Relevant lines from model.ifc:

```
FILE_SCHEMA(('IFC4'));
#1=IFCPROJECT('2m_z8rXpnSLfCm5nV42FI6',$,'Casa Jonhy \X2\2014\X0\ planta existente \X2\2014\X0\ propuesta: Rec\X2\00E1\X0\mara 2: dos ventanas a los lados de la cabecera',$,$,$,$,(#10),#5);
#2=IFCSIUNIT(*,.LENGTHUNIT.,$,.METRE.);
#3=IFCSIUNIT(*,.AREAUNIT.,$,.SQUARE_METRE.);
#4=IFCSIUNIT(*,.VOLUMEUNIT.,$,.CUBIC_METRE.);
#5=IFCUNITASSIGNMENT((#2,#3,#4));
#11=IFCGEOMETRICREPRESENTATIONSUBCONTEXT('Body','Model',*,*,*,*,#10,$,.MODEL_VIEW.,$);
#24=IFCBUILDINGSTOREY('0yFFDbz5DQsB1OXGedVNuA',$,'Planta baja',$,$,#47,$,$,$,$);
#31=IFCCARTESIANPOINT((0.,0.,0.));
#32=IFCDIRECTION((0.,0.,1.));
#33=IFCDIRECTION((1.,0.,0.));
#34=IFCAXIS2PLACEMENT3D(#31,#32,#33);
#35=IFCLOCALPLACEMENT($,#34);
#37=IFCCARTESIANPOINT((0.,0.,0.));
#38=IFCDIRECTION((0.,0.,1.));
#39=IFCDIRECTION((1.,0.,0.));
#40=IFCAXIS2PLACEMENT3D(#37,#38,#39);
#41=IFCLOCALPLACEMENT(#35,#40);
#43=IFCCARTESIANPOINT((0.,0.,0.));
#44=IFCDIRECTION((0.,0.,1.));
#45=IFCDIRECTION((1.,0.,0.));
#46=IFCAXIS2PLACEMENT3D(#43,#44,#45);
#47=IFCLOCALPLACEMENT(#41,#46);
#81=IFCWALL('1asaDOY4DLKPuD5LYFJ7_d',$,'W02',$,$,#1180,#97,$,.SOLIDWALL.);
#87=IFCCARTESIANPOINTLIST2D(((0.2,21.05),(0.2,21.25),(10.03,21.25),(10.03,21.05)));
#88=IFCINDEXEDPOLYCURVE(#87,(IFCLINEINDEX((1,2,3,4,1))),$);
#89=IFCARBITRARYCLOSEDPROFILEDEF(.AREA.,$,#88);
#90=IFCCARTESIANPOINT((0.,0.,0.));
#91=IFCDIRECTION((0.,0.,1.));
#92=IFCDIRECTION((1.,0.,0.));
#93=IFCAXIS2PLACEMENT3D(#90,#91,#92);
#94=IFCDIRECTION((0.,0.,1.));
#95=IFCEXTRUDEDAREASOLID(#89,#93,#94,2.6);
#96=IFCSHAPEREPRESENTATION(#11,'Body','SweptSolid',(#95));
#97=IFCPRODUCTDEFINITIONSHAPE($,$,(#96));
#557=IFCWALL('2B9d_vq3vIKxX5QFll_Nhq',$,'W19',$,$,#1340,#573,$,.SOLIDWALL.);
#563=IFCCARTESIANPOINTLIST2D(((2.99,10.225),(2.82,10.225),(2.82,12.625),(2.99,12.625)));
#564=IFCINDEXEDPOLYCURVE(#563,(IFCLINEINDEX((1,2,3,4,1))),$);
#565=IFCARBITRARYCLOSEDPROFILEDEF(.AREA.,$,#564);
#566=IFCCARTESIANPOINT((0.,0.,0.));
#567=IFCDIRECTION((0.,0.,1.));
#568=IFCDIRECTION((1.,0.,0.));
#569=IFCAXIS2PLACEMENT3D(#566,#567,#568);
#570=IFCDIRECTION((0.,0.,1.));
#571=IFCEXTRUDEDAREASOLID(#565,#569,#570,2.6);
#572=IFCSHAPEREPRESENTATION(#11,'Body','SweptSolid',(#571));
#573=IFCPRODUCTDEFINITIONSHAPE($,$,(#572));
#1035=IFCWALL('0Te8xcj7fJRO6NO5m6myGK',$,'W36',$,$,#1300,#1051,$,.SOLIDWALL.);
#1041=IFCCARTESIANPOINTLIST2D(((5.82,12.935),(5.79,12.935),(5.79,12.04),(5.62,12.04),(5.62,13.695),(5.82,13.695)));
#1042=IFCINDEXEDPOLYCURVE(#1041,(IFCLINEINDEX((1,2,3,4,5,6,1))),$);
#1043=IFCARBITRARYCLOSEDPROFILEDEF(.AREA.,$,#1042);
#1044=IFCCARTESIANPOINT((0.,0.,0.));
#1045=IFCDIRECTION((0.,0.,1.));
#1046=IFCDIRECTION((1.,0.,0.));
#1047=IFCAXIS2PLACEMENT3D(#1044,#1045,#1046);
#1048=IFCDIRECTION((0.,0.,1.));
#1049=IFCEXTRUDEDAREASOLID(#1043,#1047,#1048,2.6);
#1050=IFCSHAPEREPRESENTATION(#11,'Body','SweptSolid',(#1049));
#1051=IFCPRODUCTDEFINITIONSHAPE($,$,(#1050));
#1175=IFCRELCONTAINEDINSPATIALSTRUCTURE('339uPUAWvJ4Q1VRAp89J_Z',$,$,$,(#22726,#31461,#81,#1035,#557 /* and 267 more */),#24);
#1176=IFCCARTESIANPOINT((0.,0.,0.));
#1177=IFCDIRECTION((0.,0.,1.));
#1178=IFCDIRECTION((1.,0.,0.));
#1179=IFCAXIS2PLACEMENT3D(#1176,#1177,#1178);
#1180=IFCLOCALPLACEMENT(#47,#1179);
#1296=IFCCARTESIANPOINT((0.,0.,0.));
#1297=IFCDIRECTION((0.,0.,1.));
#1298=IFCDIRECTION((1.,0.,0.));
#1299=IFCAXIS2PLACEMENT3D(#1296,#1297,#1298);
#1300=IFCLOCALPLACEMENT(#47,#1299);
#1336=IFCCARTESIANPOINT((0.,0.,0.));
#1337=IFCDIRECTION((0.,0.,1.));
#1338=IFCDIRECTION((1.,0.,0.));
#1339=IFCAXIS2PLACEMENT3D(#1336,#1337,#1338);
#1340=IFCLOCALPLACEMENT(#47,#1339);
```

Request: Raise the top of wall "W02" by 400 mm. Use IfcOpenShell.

```python
import ifcopenshell
import ifcopenshell.geom
import ifcopenshell.util.representation
import ifcopenshell.util.shape

model = ifcopenshell.open("model.ifc")
settings = ifcopenshell.geom.settings()


def volume(element):
    """Net volume in cubic metres, openings subtracted."""
    shape = ifcopenshell.geom.create_shape(settings, element)
    return ifcopenshell.util.shape.get_volume(shape.geometry)


wall = model.by_guid("1asaDOY4DLKPuD5LYFJ7_d")
before = volume(wall)

body = ifcopenshell.util.representation.get_representation(wall, "Model", "Body")
solid = body.Items[0]
old_height = solid.Depth
solid.Depth += 0.4
after = volume(wall)

print(f"height {old_height:g} -> {solid.Depth:g}, volume {before:.3f} -> {after:.3f} m3")

model.write("model_v2.ifc")
```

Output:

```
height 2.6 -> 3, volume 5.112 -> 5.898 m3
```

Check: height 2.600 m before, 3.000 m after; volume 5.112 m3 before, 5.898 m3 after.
